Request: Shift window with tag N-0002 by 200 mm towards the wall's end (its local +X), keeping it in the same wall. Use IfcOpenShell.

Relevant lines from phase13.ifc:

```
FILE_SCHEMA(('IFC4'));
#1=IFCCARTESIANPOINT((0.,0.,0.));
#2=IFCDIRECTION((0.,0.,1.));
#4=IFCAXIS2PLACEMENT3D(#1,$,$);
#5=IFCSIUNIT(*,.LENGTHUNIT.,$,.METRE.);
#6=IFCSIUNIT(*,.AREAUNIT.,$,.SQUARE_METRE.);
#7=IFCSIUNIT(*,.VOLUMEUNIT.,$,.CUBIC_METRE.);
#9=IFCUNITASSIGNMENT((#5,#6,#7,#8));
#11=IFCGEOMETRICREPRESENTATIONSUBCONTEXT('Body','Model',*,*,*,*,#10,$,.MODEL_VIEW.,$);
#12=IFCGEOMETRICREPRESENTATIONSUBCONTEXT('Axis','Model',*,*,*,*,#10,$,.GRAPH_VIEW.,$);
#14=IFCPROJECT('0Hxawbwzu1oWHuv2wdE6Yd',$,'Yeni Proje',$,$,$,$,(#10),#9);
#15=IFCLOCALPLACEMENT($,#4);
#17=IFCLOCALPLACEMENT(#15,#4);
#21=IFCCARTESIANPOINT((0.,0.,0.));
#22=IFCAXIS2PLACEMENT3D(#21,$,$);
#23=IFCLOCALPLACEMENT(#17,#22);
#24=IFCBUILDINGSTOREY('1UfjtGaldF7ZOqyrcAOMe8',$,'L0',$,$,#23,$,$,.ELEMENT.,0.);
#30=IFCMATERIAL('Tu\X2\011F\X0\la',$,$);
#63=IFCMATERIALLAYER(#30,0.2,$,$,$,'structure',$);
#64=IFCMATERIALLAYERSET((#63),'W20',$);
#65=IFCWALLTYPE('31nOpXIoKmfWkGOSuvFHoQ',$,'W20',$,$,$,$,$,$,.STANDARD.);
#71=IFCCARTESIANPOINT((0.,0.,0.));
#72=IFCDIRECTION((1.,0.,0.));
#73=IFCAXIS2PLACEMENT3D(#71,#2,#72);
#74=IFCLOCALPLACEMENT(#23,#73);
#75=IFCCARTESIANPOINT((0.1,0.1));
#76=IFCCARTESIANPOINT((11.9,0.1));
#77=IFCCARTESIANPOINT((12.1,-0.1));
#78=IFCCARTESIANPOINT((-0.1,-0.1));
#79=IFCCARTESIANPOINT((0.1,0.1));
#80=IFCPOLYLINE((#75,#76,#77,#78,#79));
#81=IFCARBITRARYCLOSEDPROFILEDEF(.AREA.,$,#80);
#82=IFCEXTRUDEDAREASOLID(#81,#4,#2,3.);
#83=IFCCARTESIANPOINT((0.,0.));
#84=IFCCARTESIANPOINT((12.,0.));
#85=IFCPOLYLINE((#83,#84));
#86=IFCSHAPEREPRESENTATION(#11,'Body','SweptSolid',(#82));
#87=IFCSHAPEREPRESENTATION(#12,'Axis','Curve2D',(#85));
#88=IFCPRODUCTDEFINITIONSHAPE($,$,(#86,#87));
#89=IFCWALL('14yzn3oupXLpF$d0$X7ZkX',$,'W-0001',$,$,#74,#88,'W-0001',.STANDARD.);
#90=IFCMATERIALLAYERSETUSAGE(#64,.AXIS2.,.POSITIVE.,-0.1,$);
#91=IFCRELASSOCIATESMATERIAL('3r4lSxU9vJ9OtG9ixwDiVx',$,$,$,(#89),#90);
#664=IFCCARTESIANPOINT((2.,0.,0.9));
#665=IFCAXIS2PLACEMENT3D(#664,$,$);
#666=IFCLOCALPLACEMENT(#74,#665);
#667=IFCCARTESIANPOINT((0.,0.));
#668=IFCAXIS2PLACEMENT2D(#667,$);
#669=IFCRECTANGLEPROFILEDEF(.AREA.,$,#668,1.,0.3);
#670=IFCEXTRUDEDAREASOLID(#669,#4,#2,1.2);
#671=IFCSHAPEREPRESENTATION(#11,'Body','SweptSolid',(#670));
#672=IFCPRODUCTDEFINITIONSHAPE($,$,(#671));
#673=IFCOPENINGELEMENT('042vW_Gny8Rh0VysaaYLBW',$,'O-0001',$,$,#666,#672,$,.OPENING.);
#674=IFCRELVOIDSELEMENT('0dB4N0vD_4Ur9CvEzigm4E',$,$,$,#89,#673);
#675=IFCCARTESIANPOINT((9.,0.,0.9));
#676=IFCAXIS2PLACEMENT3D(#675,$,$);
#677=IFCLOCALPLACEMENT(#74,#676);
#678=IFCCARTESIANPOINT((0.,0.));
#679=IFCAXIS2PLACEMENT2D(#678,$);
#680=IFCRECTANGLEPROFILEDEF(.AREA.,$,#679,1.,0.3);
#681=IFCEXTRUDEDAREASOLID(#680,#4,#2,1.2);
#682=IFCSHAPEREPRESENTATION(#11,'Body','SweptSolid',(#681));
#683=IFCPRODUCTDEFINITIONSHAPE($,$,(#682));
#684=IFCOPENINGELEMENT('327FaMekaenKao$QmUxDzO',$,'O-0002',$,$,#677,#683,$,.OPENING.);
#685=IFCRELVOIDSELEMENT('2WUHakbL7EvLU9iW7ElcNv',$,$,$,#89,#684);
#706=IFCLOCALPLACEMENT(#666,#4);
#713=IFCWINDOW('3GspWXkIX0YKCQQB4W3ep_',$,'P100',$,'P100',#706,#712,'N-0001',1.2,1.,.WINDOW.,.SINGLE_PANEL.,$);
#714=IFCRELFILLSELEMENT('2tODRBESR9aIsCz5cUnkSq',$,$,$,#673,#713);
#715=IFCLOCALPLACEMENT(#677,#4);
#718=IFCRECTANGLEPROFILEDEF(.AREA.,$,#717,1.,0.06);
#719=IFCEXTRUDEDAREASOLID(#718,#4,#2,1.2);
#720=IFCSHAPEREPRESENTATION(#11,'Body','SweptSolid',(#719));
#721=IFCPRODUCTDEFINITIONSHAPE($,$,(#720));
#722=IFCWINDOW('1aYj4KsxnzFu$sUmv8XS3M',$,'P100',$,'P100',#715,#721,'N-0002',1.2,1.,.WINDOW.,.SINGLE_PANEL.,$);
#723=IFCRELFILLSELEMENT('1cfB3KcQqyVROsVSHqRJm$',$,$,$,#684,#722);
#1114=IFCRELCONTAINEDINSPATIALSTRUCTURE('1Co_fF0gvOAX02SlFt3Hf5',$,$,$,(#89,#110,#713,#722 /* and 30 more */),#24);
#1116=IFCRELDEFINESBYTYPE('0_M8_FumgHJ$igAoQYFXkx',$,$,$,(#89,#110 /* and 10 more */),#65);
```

```python
import ifcopenshell
import ifcopenshell.api.geometry
import ifcopenshell.util.placement
import ifcopenshell.util.unit

model = ifcopenshell.open("phase13.ifc")
unit_scale = ifcopenshell.util.unit.calculate_unit_scale(model)

window = model.by_id(722)
opening = window.FillsVoids[0].RelatingOpeningElement
wall = opening.VoidsElements[0].RelatingBuildingElement

wall_matrix = ifcopenshell.util.placement.get_local_placement(wall.ObjectPlacement)
shift = wall_matrix[:3, 0] * 0.2 / unit_scale
before = ifcopenshell.util.placement.get_local_placement(window.ObjectPlacement)[:3, 3].copy()

# The window is placed relative to its opening, so it follows when the opening moves.
matrix = ifcopenshell.util.placement.get_local_placement(opening.ObjectPlacement)
matrix[:3, 3] += shift
ifcopenshell.api.geometry.edit_object_placement(
    model, product=opening, matrix=matrix, is_si=False, should_transform_children=True
)

after = ifcopenshell.util.placement.get_local_placement(window.ObjectPlacement)[:3, 3]
print("window moved by", (after - before).round(3) + 0.0)

model.write("phase13-out.ifc")
```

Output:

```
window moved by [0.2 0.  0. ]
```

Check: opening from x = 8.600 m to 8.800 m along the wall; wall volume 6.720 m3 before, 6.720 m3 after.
